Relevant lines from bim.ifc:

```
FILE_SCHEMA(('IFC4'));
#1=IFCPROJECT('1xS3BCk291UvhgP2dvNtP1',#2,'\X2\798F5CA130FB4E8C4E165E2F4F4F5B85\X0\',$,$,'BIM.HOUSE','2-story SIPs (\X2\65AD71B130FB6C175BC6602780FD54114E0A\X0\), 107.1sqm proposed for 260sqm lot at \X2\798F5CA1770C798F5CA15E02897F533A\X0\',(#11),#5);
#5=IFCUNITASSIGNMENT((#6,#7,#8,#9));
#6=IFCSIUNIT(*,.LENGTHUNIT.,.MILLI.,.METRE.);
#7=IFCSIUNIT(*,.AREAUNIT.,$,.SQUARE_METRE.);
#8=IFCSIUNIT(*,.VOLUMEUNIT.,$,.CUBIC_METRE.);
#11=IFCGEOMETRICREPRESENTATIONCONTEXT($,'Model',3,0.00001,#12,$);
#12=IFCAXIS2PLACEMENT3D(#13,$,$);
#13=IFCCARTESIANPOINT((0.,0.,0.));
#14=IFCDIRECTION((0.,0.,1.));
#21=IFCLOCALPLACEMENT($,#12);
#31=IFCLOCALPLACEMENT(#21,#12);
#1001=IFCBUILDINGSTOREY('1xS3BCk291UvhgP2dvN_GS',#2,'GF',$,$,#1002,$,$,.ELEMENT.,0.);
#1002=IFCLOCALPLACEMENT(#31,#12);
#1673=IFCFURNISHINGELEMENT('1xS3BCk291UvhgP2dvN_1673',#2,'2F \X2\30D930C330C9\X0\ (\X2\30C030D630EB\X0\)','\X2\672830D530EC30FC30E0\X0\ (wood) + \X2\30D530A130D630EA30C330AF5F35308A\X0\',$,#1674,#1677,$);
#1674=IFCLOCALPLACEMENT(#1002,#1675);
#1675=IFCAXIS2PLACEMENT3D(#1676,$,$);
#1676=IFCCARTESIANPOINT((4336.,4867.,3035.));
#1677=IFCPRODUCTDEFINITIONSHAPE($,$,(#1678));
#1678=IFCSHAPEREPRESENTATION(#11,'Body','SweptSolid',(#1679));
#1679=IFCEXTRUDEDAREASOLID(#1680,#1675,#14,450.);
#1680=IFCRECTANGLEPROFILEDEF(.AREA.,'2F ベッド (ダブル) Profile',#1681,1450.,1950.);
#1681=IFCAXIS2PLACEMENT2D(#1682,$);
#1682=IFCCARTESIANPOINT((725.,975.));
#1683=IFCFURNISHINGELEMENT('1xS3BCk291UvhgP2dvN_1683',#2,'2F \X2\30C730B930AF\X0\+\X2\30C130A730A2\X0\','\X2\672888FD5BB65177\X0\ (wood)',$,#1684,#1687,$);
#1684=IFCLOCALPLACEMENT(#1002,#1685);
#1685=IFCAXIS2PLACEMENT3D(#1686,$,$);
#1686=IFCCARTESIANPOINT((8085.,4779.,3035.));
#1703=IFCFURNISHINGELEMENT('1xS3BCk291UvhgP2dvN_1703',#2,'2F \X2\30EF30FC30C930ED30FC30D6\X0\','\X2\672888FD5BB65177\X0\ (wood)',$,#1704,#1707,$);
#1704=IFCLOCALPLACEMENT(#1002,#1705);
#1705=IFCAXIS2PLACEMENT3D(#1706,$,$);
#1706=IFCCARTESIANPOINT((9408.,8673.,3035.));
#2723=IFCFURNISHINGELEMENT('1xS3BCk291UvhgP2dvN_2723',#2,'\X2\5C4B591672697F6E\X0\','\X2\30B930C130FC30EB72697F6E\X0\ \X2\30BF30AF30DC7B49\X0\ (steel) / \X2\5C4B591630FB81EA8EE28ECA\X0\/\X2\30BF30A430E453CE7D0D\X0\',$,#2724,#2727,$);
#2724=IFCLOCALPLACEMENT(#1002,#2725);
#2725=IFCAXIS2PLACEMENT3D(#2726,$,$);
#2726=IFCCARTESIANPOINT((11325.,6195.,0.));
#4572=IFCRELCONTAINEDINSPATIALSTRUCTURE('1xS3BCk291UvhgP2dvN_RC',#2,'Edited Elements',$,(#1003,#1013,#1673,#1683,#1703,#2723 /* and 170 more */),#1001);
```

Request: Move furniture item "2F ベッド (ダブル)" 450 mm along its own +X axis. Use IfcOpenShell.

```python
import ifcopenshell
import ifcopenshell.api.geometry
import ifcopenshell.util.placement

model = ifcopenshell.open("bim.ifc")

item = model.by_guid("1xS3BCk291UvhgP2dvN_1673")
matrix = ifcopenshell.util.placement.get_local_placement(item.ObjectPlacement)
matrix[:3, 3] += matrix[:3, 0] * 450.0
ifcopenshell.api.geometry.edit_object_placement(model, product=item, matrix=matrix, is_si=False)

print(ifcopenshell.util.placement.get_local_placement(item.ObjectPlacement).round(3) + 0.0)

model.write("bim-out.ifc")
```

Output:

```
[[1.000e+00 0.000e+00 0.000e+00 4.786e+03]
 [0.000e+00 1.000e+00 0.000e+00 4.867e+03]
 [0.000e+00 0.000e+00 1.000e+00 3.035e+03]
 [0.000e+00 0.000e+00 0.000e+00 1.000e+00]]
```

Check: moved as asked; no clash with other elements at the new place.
